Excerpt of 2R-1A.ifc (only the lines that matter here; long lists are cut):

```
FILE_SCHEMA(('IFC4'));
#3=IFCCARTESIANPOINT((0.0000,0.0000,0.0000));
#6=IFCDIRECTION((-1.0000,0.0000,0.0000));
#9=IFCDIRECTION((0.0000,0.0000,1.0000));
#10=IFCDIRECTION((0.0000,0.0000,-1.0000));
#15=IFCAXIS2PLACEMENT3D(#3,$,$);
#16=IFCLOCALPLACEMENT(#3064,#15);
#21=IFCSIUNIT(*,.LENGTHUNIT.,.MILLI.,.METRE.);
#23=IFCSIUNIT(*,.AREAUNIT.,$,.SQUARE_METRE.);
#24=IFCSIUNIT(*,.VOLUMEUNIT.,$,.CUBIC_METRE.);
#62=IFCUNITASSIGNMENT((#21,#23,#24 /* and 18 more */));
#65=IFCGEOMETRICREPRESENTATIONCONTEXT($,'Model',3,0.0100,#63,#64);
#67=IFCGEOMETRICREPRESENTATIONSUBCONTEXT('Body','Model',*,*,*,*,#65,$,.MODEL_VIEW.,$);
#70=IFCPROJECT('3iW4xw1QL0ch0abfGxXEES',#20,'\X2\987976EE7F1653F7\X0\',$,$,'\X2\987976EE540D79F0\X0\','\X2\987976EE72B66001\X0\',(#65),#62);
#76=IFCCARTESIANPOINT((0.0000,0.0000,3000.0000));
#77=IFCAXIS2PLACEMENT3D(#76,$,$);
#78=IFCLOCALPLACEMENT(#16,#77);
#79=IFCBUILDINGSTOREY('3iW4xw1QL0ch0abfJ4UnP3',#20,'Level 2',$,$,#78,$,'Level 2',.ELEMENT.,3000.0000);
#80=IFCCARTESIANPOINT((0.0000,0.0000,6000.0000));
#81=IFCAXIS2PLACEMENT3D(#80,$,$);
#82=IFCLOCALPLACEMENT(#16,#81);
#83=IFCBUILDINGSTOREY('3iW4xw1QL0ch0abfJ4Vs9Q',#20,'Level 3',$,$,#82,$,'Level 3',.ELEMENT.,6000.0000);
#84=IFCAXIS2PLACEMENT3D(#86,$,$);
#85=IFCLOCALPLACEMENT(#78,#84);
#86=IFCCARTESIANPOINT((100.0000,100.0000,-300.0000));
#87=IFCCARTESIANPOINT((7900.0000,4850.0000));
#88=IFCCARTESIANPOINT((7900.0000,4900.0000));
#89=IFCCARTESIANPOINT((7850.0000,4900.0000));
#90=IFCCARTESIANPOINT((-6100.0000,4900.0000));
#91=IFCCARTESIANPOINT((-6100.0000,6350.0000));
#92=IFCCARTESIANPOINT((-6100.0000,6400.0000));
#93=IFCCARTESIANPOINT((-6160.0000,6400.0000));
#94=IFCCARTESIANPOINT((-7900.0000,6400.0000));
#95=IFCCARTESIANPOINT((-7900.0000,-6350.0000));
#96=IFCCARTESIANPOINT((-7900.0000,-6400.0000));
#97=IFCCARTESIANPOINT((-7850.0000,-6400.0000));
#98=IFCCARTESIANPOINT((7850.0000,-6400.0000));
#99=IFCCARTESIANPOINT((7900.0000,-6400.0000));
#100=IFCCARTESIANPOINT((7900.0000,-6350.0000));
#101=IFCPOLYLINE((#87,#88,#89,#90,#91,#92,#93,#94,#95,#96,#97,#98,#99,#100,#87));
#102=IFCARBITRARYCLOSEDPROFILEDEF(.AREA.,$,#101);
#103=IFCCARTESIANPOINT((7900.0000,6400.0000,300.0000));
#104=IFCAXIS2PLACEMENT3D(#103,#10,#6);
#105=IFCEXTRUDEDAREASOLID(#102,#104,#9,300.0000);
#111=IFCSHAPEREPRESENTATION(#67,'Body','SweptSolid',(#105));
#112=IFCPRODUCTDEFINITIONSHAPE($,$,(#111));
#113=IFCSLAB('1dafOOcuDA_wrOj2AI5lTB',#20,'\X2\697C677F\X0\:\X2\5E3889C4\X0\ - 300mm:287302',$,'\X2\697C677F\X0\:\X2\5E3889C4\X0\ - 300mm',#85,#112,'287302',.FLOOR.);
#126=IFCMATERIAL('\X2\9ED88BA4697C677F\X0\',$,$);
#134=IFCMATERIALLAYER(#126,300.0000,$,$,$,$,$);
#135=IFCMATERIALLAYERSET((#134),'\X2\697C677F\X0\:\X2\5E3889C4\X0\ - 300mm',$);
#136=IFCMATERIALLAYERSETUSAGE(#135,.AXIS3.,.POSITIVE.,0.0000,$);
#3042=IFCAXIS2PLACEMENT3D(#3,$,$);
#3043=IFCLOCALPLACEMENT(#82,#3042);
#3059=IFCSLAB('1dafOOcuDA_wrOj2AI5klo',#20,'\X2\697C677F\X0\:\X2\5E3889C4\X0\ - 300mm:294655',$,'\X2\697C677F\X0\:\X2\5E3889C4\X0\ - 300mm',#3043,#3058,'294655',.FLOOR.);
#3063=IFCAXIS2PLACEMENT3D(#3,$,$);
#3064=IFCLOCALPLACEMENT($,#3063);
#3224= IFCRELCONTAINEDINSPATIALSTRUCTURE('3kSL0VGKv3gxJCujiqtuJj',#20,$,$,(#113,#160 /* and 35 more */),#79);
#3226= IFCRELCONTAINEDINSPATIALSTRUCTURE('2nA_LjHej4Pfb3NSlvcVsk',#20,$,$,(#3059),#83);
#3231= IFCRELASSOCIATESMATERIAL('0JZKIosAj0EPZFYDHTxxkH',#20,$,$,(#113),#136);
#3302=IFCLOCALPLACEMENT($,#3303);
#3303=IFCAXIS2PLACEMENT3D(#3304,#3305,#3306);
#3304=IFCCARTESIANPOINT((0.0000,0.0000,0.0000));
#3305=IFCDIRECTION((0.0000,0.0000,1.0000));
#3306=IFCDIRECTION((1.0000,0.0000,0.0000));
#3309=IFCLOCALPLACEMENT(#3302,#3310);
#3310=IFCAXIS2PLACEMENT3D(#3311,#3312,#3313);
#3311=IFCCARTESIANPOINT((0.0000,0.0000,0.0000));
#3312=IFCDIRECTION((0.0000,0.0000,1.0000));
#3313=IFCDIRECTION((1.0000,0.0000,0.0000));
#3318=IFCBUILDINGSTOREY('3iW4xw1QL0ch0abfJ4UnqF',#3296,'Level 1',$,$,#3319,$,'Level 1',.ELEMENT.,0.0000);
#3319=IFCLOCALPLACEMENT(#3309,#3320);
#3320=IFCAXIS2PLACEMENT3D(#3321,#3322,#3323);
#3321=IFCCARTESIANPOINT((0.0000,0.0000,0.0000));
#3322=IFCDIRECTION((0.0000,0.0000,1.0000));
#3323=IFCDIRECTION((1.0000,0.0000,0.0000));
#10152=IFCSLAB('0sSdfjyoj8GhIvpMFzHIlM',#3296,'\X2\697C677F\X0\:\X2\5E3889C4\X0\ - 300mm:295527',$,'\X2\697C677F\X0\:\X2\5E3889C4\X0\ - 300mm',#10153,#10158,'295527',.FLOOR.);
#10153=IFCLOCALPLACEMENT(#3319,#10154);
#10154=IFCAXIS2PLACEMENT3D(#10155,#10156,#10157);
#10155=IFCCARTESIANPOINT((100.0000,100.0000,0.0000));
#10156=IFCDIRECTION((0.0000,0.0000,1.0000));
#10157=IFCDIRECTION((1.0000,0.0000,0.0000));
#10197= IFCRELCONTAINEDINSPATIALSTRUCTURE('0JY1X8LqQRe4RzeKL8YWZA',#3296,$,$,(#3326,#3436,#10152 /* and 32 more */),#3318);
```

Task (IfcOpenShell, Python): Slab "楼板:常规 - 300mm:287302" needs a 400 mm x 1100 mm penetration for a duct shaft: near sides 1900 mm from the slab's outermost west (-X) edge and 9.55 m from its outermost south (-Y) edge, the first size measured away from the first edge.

```python
import numpy as np
import ifcopenshell
import ifcopenshell.api.feature
import ifcopenshell.api.geometry
import ifcopenshell.api.root
import ifcopenshell.geom
import ifcopenshell.util.placement
import ifcopenshell.util.representation
import ifcopenshell.util.shape
import ifcopenshell.util.unit

model = ifcopenshell.open("2R-1A.ifc")
unit_scale = ifcopenshell.util.unit.calculate_unit_scale(model)
settings = ifcopenshell.geom.settings()


def volume(element):
    """Net volume in cubic metres, openings subtracted."""
    shape = ifcopenshell.geom.create_shape(settings, element)
    return ifcopenshell.util.shape.get_volume(shape.geometry)


slab = model.by_guid("1dafOOcuDA_wrOj2AI5lTB")
before = volume(slab)

# Extent in the slab's own axes, in metres. The edges named are its -X and -Y sides.
slab_shape = ifcopenshell.geom.create_shape(settings, slab)
vertices = ifcopenshell.util.shape.get_vertices(slab_shape.geometry)
x_min, y_min, bottom = vertices.min(axis=0)
top = vertices[:, 2].max()

opening = ifcopenshell.api.root.create_entity(model, ifc_class="IfcOpeningElement", name="Duct shaft opening", predefined_type="OPENING")
context = ifcopenshell.util.representation.get_context(model, "Model", "Body", "MODEL_VIEW")
width, depth = 0.4, 1.1
outline = [(0.0, 0.0), (width, 0.0), (width, depth), (0.0, depth), (0.0, 0.0)]
# Overshoot both faces by 50 mm so the cut is clean.
shape = ifcopenshell.api.geometry.add_slab_representation(
    model, context=context, depth=top - bottom + 0.1, polyline=outline
)
ifcopenshell.api.geometry.assign_representation(model, product=opening, representation=shape)

matrix = ifcopenshell.util.placement.get_local_placement(slab.ObjectPlacement)
matrix[:, 3] = matrix @ np.append(np.array([x_min + 1.9, y_min + 9.55, bottom - 0.05]) / unit_scale, 1.0)
ifcopenshell.api.geometry.edit_object_placement(model, product=opening, matrix=matrix, is_si=False)
ifcopenshell.api.feature.add_feature(model, feature=opening, element=slab)

after = volume(slab)

print(f"slab volume {before:.3f} -> {after:.3f} m3")

model.write("2R-1A_edited.ifc")
```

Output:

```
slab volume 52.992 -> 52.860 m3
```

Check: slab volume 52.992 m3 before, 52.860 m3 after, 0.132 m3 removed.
